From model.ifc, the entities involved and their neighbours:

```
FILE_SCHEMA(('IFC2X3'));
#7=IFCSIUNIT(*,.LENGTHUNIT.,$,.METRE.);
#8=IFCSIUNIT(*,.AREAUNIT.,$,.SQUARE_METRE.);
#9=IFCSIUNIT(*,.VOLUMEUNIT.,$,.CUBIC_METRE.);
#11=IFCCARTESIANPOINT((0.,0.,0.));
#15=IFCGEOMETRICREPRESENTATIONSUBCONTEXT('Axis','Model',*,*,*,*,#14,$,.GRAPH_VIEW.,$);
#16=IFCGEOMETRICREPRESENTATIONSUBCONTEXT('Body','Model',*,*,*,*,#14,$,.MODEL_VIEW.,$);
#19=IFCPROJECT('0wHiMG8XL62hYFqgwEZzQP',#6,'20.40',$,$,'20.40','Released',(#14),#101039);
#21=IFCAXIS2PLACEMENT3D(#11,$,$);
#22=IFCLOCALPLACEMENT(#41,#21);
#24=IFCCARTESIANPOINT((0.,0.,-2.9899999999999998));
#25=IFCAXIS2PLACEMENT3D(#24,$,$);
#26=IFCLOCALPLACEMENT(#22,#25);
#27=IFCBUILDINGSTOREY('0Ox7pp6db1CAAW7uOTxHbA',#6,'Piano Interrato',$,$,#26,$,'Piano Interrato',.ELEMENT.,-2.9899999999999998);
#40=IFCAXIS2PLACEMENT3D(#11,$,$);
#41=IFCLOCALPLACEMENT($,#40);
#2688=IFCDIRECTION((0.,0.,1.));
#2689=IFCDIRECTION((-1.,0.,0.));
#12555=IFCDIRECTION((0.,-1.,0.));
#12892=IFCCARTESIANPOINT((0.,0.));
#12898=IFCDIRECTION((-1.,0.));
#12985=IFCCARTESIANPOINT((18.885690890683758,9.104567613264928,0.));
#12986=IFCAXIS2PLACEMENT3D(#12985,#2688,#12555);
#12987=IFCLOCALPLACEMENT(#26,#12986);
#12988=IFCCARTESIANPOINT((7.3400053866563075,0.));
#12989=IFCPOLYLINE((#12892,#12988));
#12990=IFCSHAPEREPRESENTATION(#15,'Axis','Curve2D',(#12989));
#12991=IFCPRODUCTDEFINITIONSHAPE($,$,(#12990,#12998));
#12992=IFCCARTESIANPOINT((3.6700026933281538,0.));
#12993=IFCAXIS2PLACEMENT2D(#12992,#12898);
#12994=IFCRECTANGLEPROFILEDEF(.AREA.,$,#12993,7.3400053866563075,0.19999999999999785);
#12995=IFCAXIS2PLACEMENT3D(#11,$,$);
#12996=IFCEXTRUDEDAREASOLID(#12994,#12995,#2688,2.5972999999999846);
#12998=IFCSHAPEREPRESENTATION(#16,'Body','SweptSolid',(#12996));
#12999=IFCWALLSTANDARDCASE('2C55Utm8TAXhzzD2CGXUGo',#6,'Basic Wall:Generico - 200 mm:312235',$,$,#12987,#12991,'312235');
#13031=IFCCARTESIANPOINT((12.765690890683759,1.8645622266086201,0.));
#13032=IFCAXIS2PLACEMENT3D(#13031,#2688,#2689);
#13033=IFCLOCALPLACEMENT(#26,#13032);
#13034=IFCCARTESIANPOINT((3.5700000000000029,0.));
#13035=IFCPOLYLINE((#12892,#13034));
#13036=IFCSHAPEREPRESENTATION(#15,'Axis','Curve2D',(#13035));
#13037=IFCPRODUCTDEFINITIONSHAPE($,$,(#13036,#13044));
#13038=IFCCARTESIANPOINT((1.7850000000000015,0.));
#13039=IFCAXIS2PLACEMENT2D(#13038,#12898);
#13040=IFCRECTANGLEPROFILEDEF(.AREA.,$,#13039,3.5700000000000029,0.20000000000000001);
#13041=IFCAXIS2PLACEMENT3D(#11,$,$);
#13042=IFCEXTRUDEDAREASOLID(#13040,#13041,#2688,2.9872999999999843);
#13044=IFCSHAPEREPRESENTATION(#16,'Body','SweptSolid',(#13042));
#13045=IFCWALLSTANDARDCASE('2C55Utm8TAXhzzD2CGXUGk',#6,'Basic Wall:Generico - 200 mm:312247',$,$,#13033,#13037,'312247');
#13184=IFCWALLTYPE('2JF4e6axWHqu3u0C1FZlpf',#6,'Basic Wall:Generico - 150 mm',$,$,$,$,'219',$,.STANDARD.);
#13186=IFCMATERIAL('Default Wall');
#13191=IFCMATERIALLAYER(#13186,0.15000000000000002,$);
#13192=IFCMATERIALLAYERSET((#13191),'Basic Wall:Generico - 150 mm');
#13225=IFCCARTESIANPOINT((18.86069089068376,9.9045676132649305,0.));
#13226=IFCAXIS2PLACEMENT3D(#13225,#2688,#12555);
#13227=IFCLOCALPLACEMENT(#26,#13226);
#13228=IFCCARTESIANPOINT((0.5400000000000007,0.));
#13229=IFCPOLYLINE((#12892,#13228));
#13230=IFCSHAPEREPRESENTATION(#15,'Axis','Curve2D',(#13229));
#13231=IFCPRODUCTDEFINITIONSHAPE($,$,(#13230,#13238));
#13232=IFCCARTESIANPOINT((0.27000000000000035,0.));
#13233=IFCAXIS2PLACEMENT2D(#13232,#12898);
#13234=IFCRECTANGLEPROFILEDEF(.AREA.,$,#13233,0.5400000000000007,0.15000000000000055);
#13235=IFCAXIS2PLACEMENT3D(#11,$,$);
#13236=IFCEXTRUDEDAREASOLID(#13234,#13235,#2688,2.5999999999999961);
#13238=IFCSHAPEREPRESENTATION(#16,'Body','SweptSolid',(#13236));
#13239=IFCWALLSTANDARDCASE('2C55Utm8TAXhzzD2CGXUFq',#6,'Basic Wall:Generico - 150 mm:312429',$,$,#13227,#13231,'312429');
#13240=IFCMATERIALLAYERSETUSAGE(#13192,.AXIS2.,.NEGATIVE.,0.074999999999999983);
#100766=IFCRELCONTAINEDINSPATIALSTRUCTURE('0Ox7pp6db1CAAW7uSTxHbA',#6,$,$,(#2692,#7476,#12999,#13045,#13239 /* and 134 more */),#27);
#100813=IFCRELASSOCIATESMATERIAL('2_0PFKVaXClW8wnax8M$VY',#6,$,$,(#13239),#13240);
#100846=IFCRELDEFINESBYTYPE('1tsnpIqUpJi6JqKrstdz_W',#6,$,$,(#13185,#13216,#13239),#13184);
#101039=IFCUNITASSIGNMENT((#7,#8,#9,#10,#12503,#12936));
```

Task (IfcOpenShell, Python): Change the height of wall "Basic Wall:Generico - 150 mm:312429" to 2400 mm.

```python
import ifcopenshell
import ifcopenshell.geom
import ifcopenshell.util.representation
import ifcopenshell.util.shape
import ifcopenshell.util.unit

model = ifcopenshell.open("model.ifc")
unit_scale = ifcopenshell.util.unit.calculate_unit_scale(model)
settings = ifcopenshell.geom.settings()


def volume(element):
    """Net volume in cubic metres, openings subtracted."""
    shape = ifcopenshell.geom.create_shape(settings, element)
    return ifcopenshell.util.shape.get_volume(shape.geometry)


wall = model.by_id(13239)
before = volume(wall)

body = ifcopenshell.util.representation.get_representation(wall, "Model", "Body")
solid = body.Items[0]
old_height = solid.Depth
solid.Depth = 2.4 / unit_scale
after = volume(wall)

print(f"height {old_height:g} -> {solid.Depth:g}, volume {before:.3f} -> {after:.3f} m3")

model.write("model_updated.ifc")
```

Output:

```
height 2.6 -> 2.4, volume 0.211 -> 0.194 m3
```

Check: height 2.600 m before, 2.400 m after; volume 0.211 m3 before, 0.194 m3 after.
